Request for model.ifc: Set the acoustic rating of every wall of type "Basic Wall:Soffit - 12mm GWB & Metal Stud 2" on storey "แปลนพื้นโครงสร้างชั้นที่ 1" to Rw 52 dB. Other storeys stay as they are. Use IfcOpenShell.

First a look at what the model holds.

```python
import ifcopenshell
import ifcopenshell.util.element

model = ifcopenshell.open("model.ifc")
print(model.schema)
storey = next(s for s in model.by_type("IfcBuildingStorey") if s.Name == "แปลนพื้นโครงสร้างชั้นที่ 1")
walls = [e for e in ifcopenshell.util.element.get_decomposition(storey) if e.is_a("IfcWall")]
seen = {}
for e in walls:
    element_type = ifcopenshell.util.element.get_type(e)
    key = (element_type.Name if element_type != e and element_type else None, ifcopenshell.util.element.get_pset(e, "Pset_WallCommon", "AcousticRating"))
    seen[key] = seen.get(key, 0) + 1
for (name, value), count in sorted(seen.items(), key=str):
    print(count, "x", name, "|", value)
```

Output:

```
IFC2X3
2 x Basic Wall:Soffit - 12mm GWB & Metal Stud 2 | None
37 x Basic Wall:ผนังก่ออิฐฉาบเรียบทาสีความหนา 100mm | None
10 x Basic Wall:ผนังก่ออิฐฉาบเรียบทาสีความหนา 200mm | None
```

```python
import ifcopenshell
import ifcopenshell.api.pset
import ifcopenshell.util.element

model = ifcopenshell.open("model.ifc")

storey = next(s for s in model.by_type("IfcBuildingStorey") if s.Name == "แปลนพื้นโครงสร้างชั้นที่ 1")
walls = [e for e in ifcopenshell.util.element.get_decomposition(storey) if e.is_a("IfcWall")]

count = 0
for e in walls:
    element_type = ifcopenshell.util.element.get_type(e)
    if element_type in (None, e) or element_type.Name != "Basic Wall:Soffit - 12mm GWB & Metal Stud 2":
        continue
    # add_pset returns the element's existing set when there is one.
    pset = ifcopenshell.api.pset.add_pset(model, product=e, name="Pset_WallCommon")
    ifcopenshell.api.pset.edit_pset(model, pset=pset, properties={"AcousticRating": "Rw 52 dB"})
    count += 1

print(count, "walls updated")

model.write("model_v2.ifc")
```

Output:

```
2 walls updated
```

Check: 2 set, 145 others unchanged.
